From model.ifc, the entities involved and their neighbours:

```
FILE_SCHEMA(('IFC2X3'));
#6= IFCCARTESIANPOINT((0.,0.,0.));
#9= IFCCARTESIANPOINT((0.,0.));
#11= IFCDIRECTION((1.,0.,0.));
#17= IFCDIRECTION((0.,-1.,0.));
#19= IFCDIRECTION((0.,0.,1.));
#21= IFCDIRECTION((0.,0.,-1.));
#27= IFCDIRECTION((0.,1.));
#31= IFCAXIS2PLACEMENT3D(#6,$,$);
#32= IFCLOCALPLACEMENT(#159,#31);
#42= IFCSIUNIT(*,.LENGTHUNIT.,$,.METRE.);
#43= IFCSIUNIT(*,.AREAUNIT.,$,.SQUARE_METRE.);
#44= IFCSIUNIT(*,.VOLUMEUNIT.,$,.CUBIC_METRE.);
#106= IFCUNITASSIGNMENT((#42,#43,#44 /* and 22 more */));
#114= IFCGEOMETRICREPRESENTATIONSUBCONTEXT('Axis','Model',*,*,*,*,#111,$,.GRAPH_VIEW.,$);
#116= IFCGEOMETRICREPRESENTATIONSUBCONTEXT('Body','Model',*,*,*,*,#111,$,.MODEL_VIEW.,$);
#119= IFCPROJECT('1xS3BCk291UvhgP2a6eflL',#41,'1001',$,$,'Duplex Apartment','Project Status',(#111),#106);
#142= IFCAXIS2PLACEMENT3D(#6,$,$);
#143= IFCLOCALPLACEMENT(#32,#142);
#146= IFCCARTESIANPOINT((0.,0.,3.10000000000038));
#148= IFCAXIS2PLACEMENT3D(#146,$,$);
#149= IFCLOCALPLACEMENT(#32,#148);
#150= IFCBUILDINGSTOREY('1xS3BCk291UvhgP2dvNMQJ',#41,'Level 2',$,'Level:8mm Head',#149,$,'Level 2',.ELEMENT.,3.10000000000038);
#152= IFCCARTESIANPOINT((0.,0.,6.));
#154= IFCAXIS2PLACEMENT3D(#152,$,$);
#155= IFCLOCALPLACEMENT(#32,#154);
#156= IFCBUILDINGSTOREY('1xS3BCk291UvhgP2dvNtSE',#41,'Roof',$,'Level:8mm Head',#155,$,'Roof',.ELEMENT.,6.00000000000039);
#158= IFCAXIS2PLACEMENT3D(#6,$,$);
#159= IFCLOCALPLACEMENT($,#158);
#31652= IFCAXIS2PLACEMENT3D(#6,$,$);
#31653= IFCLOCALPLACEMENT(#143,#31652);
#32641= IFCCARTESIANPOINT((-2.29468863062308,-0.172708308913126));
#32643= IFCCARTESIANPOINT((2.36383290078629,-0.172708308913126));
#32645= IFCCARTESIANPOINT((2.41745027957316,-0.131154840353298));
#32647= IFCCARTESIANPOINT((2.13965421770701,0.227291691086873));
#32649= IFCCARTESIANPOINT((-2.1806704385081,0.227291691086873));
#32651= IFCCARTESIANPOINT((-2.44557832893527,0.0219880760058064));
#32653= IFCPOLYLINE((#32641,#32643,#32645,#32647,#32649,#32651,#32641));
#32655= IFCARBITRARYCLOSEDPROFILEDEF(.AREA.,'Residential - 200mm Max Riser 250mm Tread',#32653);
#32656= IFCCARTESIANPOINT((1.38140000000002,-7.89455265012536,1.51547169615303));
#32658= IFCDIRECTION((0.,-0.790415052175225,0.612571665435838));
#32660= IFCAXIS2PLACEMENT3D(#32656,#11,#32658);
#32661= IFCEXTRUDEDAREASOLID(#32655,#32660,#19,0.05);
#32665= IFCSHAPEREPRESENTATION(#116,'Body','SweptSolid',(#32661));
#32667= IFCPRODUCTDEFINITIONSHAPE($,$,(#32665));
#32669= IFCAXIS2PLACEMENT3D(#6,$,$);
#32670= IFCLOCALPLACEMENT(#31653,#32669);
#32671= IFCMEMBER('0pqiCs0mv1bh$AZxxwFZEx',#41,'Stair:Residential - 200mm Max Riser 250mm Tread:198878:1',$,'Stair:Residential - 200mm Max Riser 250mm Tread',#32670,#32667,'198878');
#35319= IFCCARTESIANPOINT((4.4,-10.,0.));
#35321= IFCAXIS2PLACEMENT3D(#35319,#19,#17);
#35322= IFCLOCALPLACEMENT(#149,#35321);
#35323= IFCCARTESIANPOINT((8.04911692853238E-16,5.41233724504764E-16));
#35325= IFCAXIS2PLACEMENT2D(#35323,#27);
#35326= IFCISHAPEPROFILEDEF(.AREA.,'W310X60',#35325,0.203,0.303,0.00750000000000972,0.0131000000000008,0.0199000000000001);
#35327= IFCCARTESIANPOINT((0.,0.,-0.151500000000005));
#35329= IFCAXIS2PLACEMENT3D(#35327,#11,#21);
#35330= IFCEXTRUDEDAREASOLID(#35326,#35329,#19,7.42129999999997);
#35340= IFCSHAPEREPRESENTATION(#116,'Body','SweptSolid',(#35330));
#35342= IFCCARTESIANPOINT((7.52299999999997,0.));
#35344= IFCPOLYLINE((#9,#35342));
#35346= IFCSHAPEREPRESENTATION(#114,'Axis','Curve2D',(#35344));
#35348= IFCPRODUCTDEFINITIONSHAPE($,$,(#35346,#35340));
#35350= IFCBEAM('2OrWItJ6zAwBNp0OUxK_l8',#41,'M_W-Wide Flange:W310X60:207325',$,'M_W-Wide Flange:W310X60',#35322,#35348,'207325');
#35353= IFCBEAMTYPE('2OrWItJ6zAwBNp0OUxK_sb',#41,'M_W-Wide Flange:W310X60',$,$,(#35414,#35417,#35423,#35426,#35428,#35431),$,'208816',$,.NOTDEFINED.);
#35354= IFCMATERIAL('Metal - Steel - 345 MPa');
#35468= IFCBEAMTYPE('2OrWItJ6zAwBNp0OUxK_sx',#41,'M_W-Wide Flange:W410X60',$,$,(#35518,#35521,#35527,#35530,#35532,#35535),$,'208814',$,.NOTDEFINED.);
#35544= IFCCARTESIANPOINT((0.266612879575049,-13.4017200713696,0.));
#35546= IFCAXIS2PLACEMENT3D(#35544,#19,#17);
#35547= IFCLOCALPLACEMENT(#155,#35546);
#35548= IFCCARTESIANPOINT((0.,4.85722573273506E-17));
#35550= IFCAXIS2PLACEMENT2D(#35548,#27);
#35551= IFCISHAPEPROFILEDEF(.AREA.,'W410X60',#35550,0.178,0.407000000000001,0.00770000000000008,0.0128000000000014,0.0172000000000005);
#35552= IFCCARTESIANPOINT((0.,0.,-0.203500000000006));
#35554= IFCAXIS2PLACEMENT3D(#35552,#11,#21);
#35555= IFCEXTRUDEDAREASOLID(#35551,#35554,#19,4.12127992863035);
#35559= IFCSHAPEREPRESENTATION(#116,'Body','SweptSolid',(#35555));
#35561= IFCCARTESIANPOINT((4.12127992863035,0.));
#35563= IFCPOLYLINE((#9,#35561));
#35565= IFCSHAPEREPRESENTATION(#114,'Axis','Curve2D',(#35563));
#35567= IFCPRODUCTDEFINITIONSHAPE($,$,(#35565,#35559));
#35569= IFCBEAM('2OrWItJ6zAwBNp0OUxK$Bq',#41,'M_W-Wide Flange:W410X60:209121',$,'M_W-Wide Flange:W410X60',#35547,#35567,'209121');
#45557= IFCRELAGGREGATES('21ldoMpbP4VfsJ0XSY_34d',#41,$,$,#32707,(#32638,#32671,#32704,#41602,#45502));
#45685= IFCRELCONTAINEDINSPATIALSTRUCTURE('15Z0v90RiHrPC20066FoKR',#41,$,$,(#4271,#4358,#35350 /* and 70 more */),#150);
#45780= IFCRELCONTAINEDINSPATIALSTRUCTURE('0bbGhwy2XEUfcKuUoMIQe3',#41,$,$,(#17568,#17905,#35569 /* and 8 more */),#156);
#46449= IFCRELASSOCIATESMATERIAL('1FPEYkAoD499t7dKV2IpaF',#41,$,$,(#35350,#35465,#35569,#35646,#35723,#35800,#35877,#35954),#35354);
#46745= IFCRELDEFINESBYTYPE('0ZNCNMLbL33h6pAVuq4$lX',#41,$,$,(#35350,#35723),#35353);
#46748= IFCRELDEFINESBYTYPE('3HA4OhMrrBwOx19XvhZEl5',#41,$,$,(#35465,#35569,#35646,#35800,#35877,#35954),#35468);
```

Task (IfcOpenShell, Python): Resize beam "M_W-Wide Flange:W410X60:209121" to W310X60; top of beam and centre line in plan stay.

```python
import ifcopenshell
import ifcopenshell.api.type
import ifcopenshell.util.element
import ifcopenshell.util.representation

model = ifcopenshell.open("model.ifc")

member = model.by_guid("2OrWItJ6zAwBNp0OUxK$Bq")
source = next(p for p in model.by_type("IfcIShapeProfileDef") if p.ProfileName == "W310X60")

body = ifcopenshell.util.representation.get_representation(member, "Model", "Body")
solid = body.Items[0]
old_profile = solid.SweptArea

# Copy the section's sizes but keep this member's own profile position.
profile = ifcopenshell.util.element.copy(model, source)
# Profiles are centred, so shift by half the change in depth to hold the top.
shift = (old_profile.OverallDepth - profile.OverallDepth) / 2
x, y = old_profile.Position.Location.Coordinates
up = (-1.0, 0.0)  # upwards, in the solid's own plane
location = model.createIfcCartesianPoint((x + up[0] * shift, y + up[1] * shift))
profile.Position = model.createIfcAxis2Placement2D(location, old_profile.Position.RefDirection)
solid.SweptArea = profile
if not model.get_total_inverses(old_profile):
    ifcopenshell.util.element.remove_deep2(model, old_profile)

new_type = model.by_guid("2OrWItJ6zAwBNp0OUxK_sb")
ifcopenshell.api.type.assign_type(
    model, related_objects=[member], relating_type=new_type, should_map_representations=False
)
member.Name = member.Name.replace("W410X60", "W310X60")
member.ObjectType = "M_W-Wide Flange:W310X60"

print(solid.SweptArea)

model.write("model_edited.ifc")
```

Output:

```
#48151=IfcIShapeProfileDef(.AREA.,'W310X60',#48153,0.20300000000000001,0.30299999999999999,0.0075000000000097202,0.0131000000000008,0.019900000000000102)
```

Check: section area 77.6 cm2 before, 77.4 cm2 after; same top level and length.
